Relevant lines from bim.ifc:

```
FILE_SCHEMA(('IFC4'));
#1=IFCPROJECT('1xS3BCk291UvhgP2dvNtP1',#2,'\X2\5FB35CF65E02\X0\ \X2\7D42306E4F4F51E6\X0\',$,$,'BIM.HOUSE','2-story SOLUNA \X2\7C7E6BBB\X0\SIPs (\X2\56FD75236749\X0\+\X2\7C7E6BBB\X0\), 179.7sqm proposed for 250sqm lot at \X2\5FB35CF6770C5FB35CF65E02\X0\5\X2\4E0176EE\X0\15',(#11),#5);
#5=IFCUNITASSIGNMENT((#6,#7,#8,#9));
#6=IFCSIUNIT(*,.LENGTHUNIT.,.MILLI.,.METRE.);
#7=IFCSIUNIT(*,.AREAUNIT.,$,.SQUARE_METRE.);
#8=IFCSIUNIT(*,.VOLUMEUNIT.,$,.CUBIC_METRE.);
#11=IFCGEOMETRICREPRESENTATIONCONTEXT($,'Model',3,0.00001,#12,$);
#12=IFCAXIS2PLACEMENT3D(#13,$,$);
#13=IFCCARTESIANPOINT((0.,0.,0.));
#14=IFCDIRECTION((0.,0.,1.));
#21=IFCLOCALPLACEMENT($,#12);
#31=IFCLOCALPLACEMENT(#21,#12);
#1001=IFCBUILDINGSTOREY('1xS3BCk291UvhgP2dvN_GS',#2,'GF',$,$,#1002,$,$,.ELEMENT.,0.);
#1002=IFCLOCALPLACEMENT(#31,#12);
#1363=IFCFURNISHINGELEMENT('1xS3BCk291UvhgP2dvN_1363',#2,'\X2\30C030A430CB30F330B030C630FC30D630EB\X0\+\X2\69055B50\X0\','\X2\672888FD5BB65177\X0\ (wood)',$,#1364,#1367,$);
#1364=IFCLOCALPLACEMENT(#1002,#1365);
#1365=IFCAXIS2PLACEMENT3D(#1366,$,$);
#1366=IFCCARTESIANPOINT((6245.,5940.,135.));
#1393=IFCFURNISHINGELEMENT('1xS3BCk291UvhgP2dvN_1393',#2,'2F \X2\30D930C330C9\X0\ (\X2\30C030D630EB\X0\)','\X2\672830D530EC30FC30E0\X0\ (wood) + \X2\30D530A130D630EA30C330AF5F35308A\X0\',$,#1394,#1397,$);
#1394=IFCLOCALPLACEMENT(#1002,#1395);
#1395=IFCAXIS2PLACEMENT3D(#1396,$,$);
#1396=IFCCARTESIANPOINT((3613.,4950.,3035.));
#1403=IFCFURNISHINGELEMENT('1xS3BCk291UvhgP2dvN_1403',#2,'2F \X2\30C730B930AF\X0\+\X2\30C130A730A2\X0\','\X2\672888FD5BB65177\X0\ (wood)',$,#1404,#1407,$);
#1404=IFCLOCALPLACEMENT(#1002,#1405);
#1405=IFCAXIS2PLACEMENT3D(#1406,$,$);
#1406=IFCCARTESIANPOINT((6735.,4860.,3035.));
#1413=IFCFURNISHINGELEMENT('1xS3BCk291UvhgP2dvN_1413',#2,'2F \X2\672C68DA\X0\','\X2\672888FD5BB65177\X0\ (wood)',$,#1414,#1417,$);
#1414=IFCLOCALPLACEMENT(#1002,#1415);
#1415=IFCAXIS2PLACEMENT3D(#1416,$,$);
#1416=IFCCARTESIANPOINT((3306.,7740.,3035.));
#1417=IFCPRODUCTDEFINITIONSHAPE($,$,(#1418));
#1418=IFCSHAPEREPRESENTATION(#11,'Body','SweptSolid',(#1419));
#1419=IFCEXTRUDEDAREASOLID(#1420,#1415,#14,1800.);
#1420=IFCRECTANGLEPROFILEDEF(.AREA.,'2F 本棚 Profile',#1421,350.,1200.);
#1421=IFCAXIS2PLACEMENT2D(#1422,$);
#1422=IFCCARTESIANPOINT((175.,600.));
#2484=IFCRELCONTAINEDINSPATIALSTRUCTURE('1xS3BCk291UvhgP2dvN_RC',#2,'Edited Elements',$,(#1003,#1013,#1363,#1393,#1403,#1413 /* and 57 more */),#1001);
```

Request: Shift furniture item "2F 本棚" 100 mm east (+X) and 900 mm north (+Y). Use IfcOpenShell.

```python
import ifcopenshell
import ifcopenshell.api.geometry
import ifcopenshell.util.placement
import ifcopenshell.util.unit

model = ifcopenshell.open("bim.ifc")
unit_scale = ifcopenshell.util.unit.calculate_unit_scale(model)

item = model.by_id(1413)
matrix = ifcopenshell.util.placement.get_local_placement(item.ObjectPlacement)
matrix[0, 3] += 0.1 / unit_scale
matrix[1, 3] += 0.9 / unit_scale
ifcopenshell.api.geometry.edit_object_placement(model, product=item, matrix=matrix, is_si=False)

print(ifcopenshell.util.placement.get_local_placement(item.ObjectPlacement).round(3) + 0.0)

model.write("bim-out.ifc")
```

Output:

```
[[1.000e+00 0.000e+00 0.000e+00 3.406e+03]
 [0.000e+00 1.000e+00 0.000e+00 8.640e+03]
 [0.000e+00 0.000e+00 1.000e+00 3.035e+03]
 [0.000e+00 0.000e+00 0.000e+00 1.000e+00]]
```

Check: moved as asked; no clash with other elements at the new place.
